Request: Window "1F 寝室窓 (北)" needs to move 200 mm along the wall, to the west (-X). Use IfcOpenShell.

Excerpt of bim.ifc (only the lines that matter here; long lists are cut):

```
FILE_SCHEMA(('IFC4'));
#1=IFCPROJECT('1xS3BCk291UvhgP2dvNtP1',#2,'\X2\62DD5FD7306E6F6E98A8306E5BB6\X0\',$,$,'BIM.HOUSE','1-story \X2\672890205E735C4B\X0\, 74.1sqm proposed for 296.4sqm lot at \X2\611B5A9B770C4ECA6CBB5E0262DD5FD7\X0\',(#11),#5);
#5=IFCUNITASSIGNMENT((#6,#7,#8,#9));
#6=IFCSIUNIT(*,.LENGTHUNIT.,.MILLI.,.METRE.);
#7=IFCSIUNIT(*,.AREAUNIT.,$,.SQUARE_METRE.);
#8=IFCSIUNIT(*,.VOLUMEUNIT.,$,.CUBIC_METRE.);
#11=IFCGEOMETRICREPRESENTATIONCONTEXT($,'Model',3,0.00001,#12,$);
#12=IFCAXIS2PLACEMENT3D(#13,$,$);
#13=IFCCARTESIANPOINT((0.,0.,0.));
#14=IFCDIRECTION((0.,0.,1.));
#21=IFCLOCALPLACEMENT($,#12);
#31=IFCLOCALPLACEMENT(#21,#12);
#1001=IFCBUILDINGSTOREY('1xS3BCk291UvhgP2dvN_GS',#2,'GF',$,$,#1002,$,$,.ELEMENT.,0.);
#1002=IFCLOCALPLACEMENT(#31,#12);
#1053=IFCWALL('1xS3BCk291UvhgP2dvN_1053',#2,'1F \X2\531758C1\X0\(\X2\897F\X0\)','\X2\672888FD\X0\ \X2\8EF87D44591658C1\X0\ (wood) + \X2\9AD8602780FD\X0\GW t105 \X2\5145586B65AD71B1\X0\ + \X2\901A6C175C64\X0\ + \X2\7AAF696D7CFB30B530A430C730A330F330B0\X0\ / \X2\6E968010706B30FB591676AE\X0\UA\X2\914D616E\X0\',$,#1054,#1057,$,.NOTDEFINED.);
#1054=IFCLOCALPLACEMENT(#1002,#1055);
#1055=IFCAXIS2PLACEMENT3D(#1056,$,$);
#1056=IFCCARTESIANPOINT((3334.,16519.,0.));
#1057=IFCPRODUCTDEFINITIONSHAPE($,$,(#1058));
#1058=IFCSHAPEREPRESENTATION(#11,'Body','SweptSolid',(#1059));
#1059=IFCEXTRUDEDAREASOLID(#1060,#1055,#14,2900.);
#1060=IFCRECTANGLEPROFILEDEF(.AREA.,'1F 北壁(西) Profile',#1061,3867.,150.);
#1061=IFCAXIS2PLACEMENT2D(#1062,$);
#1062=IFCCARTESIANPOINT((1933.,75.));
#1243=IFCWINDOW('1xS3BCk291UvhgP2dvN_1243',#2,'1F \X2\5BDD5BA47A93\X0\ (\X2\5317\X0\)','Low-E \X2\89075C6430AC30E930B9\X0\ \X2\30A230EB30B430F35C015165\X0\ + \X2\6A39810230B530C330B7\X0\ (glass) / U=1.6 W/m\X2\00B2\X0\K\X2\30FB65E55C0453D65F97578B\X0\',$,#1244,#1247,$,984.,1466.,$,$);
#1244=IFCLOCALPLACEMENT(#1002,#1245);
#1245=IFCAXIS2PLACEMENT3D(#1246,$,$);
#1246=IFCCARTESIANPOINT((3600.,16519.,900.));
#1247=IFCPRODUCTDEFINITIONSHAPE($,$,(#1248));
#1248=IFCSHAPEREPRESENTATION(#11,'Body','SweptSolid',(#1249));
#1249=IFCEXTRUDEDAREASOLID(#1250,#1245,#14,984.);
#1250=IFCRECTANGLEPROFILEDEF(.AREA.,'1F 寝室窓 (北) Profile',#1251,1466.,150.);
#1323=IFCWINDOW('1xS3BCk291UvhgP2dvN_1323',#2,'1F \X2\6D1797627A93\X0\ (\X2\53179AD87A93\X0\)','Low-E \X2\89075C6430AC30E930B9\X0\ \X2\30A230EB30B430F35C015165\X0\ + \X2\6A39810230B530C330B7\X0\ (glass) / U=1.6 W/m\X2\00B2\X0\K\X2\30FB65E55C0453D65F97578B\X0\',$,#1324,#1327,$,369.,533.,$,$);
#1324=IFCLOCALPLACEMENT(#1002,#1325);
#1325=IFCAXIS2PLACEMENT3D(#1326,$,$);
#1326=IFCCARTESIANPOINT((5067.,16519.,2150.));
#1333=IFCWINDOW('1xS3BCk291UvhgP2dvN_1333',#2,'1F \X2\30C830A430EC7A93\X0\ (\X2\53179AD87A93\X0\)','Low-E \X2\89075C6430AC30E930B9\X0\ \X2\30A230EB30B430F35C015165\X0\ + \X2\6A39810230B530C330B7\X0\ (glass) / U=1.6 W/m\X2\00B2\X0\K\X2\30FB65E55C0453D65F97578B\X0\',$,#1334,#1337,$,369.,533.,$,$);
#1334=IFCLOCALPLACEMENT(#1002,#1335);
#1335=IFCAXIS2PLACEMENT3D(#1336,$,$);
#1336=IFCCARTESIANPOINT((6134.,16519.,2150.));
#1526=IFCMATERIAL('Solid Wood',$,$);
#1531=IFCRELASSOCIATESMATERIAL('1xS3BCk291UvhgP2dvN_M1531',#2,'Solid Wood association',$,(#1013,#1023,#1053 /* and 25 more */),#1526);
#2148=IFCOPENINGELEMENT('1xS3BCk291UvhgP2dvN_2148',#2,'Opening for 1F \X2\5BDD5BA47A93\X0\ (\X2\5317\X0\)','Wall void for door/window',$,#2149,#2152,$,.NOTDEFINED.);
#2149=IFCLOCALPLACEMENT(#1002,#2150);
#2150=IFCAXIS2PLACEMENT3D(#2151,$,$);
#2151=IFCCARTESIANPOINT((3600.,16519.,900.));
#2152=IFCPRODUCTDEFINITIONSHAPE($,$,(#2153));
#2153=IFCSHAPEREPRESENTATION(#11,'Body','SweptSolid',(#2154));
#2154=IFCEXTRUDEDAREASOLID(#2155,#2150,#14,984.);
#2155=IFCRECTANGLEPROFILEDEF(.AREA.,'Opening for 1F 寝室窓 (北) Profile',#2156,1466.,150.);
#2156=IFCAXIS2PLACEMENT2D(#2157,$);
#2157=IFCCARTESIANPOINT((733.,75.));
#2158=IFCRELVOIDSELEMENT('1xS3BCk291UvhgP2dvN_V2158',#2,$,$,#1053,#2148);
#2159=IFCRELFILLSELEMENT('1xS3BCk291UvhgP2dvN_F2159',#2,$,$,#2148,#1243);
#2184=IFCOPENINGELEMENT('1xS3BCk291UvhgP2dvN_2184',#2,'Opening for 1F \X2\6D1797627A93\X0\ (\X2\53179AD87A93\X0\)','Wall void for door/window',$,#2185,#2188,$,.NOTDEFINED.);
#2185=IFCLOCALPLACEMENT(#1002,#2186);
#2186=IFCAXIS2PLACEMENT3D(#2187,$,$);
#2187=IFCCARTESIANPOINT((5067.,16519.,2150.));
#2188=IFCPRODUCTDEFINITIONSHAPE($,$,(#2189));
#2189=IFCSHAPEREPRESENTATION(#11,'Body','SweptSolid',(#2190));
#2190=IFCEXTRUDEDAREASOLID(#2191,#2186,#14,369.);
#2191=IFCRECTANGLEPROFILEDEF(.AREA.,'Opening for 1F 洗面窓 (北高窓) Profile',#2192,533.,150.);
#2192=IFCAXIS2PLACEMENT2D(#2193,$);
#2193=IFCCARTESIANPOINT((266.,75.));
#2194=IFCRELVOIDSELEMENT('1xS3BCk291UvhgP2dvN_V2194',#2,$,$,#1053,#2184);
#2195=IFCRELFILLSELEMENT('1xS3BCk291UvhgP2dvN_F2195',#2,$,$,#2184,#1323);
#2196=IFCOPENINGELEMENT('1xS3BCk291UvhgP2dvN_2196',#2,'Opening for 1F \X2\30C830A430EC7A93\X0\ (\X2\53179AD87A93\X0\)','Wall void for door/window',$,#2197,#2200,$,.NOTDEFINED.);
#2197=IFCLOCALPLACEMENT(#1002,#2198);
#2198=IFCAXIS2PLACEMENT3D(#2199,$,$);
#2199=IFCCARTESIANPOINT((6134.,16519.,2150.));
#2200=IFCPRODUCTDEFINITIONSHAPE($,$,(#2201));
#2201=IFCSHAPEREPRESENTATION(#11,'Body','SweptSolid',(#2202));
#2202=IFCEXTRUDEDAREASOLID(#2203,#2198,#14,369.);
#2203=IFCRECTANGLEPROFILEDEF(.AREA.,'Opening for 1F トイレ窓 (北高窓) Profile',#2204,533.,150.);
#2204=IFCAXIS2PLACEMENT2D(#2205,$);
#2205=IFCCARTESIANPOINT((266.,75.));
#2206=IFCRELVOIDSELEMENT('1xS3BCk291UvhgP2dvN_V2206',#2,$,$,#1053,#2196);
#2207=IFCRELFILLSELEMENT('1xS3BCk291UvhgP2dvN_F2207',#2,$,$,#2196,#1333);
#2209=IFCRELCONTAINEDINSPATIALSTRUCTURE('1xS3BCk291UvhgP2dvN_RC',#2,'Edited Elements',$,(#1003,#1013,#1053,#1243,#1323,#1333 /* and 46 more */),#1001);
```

```python
import ifcopenshell
import ifcopenshell.api.geometry
import ifcopenshell.util.placement
import ifcopenshell.util.unit

model = ifcopenshell.open("bim.ifc")
unit_scale = ifcopenshell.util.unit.calculate_unit_scale(model)

window = model.by_id(1243)
opening = window.FillsVoids[0].RelatingOpeningElement
wall = opening.VoidsElements[0].RelatingBuildingElement

wall_matrix = ifcopenshell.util.placement.get_local_placement(wall.ObjectPlacement)
shift = wall_matrix[:3, 0] * -0.2 / unit_scale
before = ifcopenshell.util.placement.get_local_placement(window.ObjectPlacement)[:3, 3].copy()

# The window is not placed relative to its opening, so move both.
for product in (opening, window):
    matrix = ifcopenshell.util.placement.get_local_placement(product.ObjectPlacement)
    matrix[:3, 3] += shift
    ifcopenshell.api.geometry.edit_object_placement(model, product=product, matrix=matrix, is_si=False)

after = ifcopenshell.util.placement.get_local_placement(window.ObjectPlacement)[:3, 3]
print("window moved by", (after - before).round(3) + 0.0)

model.write("bim_updated.ifc")
```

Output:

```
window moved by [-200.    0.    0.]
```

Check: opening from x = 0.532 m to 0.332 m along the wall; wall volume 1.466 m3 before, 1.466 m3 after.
